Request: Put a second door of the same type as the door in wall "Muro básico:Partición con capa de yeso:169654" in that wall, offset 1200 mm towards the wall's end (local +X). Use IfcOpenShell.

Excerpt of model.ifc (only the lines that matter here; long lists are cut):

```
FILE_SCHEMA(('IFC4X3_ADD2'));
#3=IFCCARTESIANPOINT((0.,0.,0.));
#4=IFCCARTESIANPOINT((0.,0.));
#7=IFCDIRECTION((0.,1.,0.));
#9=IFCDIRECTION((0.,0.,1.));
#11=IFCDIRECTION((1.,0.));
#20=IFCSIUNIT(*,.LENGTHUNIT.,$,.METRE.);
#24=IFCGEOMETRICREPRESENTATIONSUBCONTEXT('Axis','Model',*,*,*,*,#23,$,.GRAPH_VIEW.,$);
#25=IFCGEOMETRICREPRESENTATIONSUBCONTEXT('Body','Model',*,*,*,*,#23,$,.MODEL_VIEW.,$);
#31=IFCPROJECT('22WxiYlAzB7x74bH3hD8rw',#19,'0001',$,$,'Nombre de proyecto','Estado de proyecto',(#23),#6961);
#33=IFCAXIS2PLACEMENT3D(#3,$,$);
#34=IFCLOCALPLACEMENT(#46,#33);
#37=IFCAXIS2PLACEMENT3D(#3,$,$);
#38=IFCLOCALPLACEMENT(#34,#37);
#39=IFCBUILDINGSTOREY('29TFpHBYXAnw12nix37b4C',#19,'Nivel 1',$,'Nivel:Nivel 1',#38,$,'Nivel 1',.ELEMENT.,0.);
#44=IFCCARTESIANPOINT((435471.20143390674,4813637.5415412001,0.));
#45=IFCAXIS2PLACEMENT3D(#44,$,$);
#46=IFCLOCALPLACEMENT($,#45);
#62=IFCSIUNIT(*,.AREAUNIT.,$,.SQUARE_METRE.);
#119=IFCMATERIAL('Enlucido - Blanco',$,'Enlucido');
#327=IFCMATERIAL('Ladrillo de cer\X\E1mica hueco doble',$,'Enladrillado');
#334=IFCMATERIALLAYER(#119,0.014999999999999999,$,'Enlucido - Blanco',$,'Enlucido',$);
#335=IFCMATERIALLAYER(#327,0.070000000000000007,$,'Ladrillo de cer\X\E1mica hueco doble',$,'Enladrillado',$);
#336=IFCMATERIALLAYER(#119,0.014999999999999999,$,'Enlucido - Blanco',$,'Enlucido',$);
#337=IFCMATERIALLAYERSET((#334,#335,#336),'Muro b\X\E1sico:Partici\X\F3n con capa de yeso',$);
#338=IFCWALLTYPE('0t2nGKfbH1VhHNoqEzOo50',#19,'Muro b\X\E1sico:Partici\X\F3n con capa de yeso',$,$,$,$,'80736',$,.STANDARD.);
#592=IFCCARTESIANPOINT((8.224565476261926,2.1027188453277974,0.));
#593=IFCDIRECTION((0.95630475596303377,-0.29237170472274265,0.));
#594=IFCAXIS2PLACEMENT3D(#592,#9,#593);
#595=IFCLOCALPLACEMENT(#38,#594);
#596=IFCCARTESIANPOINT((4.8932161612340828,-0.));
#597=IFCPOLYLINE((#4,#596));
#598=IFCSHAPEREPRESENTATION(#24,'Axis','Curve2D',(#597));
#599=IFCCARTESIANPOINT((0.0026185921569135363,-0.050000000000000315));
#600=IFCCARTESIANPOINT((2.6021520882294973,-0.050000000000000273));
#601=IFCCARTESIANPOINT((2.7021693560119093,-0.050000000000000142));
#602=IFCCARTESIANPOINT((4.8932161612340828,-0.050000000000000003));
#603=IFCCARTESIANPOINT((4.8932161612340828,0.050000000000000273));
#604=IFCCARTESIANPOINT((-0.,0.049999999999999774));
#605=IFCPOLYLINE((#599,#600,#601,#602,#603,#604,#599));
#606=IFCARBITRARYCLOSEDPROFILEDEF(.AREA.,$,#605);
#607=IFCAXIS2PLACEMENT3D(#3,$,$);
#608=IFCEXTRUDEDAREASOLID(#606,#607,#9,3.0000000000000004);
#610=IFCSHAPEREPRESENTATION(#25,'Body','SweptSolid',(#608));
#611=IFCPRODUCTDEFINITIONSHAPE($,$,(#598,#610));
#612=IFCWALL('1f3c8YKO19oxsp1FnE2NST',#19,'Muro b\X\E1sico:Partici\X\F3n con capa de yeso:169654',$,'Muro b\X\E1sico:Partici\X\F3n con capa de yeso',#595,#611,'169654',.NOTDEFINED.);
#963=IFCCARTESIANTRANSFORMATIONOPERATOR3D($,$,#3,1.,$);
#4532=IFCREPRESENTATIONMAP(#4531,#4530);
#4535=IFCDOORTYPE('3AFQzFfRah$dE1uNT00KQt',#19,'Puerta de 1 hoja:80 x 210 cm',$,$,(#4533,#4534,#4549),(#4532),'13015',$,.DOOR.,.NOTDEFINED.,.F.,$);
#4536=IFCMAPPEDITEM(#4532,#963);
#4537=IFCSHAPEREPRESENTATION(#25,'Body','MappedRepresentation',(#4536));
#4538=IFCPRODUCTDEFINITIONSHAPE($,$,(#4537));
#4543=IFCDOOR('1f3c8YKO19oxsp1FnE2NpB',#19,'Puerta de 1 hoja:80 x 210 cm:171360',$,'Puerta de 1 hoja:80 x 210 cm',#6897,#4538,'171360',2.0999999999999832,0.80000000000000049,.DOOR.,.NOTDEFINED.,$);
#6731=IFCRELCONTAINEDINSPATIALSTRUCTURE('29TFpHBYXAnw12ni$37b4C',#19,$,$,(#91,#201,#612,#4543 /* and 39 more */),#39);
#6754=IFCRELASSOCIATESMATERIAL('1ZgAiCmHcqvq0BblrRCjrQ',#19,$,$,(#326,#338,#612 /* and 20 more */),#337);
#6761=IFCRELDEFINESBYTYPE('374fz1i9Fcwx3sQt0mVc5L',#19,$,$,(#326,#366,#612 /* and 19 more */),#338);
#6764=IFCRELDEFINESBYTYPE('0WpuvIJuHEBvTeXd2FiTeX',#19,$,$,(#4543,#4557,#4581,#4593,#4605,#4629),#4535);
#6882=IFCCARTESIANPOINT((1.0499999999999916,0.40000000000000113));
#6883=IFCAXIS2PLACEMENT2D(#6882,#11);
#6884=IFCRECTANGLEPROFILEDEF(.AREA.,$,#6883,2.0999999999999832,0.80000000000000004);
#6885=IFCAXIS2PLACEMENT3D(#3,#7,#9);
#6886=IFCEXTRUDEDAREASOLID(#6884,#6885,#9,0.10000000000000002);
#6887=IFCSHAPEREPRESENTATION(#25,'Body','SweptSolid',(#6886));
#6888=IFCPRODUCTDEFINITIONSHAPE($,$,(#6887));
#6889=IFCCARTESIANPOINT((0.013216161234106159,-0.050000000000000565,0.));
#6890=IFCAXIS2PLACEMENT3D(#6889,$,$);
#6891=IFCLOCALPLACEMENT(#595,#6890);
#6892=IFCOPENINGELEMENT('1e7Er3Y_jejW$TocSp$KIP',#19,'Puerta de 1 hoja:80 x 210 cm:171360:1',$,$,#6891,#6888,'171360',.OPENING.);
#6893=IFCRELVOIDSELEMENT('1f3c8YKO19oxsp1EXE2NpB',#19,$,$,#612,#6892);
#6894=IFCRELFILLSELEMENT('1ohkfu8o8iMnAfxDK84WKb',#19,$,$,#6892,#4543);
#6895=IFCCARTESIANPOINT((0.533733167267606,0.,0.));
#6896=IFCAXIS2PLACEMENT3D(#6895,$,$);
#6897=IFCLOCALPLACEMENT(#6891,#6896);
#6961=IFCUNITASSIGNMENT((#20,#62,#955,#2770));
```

```python
import ifcopenshell
import ifcopenshell.api.feature
import ifcopenshell.api.geometry
import ifcopenshell.api.root
import ifcopenshell.geom
import ifcopenshell.util.element
import ifcopenshell.util.placement
import ifcopenshell.util.shape

model = ifcopenshell.open("model.ifc")
settings = ifcopenshell.geom.settings()


def volume(element):
    """Net volume in cubic metres, openings subtracted."""
    shape = ifcopenshell.geom.create_shape(settings, element)
    return ifcopenshell.util.shape.get_volume(shape.geometry)


def reuse_history(source, copy):
    """copy_class also copies each property set's owner history, people and application; keep the originals."""
    for rel in copy.IsDefinedBy:
        if rel.is_a("IfcRelDefinesByProperties") and (history := rel.RelatingPropertyDefinition.OwnerHistory):
            rel.RelatingPropertyDefinition.OwnerHistory = source.OwnerHistory
            ifcopenshell.util.element.remove_deep2(model, history)


door = model.by_guid("1f3c8YKO19oxsp1FnE2NpB")
opening = door.FillsVoids[0].RelatingOpeningElement
wall = opening.VoidsElements[0].RelatingBuildingElement
before = volume(wall)
shift = ifcopenshell.util.placement.get_local_placement(wall.ObjectPlacement)[:3, 0] * 1.2

# copy_class copies the void relationship, type, container and properties, but no geometry.
new_opening = ifcopenshell.api.root.copy_class(model, product=opening)
new_opening.Representation = ifcopenshell.util.element.copy_deep(
    model, opening.Representation, exclude=["IfcGeometricRepresentationContext", "IfcRepresentationMap"]
)
new_opening.Name = "Puerta de 1 hoja:80 x 210 cm"
new_opening.Tag = None
new_door = ifcopenshell.api.root.copy_class(model, product=door)
new_door.Representation = ifcopenshell.util.element.copy_deep(
    model, door.Representation, exclude=["IfcGeometricRepresentationContext", "IfcRepresentationMap"]
)
new_door.Name = "Puerta de 1 hoja:80 x 210 cm"
new_door.Tag = None
reuse_history(door, new_door)
ifcopenshell.api.feature.add_filling(model, opening=new_opening, element=new_door)

for old, new in ((opening, new_opening), (door, new_door)):
    matrix = ifcopenshell.util.placement.get_local_placement(old.ObjectPlacement)
    matrix[:3, 3] += shift
    ifcopenshell.api.geometry.edit_object_placement(model, product=new, matrix=matrix, is_si=False)

after = volume(wall)

print(f"wall volume {before:.3f} -> {after:.3f} m3")

model.write("model_v2.ifc")
```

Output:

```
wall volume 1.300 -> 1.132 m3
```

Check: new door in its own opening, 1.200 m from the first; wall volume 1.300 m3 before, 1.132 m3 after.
